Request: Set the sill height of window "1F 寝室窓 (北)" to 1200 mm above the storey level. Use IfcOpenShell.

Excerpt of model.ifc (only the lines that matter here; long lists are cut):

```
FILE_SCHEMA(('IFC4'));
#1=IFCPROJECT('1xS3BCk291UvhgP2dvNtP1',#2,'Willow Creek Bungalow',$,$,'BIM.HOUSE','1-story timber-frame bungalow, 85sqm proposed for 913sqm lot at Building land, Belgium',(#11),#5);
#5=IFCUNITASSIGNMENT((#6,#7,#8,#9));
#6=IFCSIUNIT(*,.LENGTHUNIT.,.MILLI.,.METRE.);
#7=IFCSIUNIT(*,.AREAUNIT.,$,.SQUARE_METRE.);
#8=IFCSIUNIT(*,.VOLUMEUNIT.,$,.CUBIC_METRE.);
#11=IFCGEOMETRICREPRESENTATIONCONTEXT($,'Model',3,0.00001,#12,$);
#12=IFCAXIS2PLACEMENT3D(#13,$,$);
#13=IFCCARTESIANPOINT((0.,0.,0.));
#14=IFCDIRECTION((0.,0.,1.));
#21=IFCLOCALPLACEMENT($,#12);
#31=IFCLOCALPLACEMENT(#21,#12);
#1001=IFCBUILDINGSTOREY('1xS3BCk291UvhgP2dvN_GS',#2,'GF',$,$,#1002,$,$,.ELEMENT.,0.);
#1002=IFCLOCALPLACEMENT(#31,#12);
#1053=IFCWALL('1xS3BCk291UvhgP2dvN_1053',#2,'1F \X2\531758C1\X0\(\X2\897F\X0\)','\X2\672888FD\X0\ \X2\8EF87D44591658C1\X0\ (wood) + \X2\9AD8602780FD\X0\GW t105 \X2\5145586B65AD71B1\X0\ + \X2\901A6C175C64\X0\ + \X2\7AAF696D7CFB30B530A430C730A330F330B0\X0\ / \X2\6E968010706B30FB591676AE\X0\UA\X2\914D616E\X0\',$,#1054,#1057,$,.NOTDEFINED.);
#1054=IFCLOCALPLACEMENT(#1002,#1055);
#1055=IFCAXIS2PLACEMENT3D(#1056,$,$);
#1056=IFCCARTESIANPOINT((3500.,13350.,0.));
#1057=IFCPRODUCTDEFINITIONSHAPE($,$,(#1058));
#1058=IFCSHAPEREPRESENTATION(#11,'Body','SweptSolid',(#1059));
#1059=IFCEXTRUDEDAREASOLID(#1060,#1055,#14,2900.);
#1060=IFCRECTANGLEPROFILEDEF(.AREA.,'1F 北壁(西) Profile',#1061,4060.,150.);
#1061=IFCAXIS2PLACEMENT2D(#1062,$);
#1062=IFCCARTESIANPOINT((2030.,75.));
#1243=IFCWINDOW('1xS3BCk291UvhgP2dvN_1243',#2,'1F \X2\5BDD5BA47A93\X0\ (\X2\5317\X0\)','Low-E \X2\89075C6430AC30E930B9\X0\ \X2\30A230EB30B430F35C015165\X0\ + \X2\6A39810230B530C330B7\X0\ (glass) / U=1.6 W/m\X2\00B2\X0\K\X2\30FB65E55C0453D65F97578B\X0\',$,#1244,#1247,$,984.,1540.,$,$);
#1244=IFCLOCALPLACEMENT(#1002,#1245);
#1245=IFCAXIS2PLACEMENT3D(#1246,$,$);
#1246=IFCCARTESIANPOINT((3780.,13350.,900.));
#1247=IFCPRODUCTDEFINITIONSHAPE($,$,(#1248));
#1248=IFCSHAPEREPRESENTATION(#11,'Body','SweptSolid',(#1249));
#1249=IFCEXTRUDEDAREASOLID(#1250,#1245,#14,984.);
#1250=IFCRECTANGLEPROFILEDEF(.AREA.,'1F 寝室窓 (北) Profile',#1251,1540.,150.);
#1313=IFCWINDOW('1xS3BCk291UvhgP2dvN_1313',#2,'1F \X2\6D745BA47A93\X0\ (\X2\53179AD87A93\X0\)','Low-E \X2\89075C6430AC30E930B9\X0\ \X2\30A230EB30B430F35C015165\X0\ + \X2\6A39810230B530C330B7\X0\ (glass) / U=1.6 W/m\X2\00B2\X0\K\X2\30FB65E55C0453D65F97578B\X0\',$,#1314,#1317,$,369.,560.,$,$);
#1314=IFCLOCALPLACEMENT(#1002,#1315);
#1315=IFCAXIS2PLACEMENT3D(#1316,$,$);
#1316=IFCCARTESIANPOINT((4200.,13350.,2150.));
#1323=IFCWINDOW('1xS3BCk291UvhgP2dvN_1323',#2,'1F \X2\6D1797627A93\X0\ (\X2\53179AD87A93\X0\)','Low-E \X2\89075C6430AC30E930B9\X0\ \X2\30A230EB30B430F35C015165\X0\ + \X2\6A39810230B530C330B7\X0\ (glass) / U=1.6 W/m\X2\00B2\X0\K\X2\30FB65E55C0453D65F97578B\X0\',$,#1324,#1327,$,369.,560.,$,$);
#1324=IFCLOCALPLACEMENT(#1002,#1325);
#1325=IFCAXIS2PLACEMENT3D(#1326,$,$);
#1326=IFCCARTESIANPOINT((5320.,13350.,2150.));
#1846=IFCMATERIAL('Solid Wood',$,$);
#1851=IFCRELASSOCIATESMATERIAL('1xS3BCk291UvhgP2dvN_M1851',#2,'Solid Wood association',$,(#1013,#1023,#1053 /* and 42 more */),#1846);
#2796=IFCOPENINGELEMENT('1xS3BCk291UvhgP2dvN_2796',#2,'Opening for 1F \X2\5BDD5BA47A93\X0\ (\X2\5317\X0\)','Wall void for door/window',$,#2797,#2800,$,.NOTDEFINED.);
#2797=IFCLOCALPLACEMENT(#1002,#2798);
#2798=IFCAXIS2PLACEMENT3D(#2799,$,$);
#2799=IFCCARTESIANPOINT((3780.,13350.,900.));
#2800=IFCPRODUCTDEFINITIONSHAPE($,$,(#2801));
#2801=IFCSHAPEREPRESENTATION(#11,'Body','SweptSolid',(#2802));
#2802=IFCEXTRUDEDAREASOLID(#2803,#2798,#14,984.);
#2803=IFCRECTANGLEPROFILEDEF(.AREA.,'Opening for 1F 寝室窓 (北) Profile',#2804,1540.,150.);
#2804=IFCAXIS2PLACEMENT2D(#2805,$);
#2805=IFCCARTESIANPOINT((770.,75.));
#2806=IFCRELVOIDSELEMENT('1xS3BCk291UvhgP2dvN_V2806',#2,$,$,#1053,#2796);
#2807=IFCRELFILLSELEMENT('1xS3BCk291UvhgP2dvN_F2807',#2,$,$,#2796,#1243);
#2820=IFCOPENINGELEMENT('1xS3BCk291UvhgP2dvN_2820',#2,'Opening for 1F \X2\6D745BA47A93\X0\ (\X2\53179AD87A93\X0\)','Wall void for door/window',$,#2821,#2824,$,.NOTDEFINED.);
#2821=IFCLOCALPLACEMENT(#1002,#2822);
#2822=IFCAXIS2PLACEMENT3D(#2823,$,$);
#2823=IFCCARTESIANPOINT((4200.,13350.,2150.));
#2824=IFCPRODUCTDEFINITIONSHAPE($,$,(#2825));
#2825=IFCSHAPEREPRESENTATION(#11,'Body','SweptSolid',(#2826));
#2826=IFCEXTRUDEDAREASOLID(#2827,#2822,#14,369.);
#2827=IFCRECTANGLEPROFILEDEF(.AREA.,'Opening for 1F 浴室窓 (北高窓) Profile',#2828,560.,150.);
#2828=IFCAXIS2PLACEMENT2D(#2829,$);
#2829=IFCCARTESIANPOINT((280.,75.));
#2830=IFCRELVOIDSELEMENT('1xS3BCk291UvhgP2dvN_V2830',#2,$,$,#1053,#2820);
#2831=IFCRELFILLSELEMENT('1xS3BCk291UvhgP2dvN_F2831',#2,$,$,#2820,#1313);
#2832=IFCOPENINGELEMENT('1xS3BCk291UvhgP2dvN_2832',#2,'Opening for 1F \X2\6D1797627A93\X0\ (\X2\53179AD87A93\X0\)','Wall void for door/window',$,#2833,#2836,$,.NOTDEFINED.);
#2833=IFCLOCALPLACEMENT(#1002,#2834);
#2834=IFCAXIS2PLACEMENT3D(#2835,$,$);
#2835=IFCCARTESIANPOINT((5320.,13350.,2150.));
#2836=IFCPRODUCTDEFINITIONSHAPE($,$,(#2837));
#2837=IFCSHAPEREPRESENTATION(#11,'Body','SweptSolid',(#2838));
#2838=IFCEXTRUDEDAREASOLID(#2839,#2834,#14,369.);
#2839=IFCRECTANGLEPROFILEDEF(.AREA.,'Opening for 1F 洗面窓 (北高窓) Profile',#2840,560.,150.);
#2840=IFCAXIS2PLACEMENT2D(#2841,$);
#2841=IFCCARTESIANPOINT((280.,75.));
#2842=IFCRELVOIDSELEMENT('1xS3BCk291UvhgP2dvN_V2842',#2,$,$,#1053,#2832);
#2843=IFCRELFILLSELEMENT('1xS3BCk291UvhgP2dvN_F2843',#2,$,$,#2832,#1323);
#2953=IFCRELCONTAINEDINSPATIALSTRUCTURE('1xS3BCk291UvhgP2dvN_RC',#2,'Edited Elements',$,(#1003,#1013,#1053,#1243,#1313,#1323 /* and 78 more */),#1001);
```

```python
import numpy as np
import ifcopenshell
import ifcopenshell.api.geometry
import ifcopenshell.geom
import ifcopenshell.util.element
import ifcopenshell.util.placement
import ifcopenshell.util.shape
import ifcopenshell.util.unit

model = ifcopenshell.open("model.ifc")
unit_scale = ifcopenshell.util.unit.calculate_unit_scale(model)

window = model.by_guid("1xS3BCk291UvhgP2dvN_1243")
opening = window.FillsVoids[0].RelatingOpeningElement
storey = ifcopenshell.util.element.get_container(window, ifc_class="IfcBuildingStorey")
level = ifcopenshell.util.placement.get_local_placement(storey.ObjectPlacement)[2, 3]

# The opening's origin need not be at the sill, so measure its lowest point.
shape = ifcopenshell.geom.create_shape(ifcopenshell.geom.settings(), opening)
bottom = ifcopenshell.util.shape.get_shape_bottom_elevation(shape, shape.geometry) / unit_scale
dz = level + 1200.0 - bottom

shift = np.array([0.0, 0.0, dz])
# The window is not placed relative to its opening, so move both.
for product in (opening, window):
    matrix = ifcopenshell.util.placement.get_local_placement(product.ObjectPlacement)
    matrix[:3, 3] += shift
    ifcopenshell.api.geometry.edit_object_placement(model, product=product, matrix=matrix, is_si=False)

print(f"moved by {dz * unit_scale:+.3f} m")

model.write("model_updated.ifc")
```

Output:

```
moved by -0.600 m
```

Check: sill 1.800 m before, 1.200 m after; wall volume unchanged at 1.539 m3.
